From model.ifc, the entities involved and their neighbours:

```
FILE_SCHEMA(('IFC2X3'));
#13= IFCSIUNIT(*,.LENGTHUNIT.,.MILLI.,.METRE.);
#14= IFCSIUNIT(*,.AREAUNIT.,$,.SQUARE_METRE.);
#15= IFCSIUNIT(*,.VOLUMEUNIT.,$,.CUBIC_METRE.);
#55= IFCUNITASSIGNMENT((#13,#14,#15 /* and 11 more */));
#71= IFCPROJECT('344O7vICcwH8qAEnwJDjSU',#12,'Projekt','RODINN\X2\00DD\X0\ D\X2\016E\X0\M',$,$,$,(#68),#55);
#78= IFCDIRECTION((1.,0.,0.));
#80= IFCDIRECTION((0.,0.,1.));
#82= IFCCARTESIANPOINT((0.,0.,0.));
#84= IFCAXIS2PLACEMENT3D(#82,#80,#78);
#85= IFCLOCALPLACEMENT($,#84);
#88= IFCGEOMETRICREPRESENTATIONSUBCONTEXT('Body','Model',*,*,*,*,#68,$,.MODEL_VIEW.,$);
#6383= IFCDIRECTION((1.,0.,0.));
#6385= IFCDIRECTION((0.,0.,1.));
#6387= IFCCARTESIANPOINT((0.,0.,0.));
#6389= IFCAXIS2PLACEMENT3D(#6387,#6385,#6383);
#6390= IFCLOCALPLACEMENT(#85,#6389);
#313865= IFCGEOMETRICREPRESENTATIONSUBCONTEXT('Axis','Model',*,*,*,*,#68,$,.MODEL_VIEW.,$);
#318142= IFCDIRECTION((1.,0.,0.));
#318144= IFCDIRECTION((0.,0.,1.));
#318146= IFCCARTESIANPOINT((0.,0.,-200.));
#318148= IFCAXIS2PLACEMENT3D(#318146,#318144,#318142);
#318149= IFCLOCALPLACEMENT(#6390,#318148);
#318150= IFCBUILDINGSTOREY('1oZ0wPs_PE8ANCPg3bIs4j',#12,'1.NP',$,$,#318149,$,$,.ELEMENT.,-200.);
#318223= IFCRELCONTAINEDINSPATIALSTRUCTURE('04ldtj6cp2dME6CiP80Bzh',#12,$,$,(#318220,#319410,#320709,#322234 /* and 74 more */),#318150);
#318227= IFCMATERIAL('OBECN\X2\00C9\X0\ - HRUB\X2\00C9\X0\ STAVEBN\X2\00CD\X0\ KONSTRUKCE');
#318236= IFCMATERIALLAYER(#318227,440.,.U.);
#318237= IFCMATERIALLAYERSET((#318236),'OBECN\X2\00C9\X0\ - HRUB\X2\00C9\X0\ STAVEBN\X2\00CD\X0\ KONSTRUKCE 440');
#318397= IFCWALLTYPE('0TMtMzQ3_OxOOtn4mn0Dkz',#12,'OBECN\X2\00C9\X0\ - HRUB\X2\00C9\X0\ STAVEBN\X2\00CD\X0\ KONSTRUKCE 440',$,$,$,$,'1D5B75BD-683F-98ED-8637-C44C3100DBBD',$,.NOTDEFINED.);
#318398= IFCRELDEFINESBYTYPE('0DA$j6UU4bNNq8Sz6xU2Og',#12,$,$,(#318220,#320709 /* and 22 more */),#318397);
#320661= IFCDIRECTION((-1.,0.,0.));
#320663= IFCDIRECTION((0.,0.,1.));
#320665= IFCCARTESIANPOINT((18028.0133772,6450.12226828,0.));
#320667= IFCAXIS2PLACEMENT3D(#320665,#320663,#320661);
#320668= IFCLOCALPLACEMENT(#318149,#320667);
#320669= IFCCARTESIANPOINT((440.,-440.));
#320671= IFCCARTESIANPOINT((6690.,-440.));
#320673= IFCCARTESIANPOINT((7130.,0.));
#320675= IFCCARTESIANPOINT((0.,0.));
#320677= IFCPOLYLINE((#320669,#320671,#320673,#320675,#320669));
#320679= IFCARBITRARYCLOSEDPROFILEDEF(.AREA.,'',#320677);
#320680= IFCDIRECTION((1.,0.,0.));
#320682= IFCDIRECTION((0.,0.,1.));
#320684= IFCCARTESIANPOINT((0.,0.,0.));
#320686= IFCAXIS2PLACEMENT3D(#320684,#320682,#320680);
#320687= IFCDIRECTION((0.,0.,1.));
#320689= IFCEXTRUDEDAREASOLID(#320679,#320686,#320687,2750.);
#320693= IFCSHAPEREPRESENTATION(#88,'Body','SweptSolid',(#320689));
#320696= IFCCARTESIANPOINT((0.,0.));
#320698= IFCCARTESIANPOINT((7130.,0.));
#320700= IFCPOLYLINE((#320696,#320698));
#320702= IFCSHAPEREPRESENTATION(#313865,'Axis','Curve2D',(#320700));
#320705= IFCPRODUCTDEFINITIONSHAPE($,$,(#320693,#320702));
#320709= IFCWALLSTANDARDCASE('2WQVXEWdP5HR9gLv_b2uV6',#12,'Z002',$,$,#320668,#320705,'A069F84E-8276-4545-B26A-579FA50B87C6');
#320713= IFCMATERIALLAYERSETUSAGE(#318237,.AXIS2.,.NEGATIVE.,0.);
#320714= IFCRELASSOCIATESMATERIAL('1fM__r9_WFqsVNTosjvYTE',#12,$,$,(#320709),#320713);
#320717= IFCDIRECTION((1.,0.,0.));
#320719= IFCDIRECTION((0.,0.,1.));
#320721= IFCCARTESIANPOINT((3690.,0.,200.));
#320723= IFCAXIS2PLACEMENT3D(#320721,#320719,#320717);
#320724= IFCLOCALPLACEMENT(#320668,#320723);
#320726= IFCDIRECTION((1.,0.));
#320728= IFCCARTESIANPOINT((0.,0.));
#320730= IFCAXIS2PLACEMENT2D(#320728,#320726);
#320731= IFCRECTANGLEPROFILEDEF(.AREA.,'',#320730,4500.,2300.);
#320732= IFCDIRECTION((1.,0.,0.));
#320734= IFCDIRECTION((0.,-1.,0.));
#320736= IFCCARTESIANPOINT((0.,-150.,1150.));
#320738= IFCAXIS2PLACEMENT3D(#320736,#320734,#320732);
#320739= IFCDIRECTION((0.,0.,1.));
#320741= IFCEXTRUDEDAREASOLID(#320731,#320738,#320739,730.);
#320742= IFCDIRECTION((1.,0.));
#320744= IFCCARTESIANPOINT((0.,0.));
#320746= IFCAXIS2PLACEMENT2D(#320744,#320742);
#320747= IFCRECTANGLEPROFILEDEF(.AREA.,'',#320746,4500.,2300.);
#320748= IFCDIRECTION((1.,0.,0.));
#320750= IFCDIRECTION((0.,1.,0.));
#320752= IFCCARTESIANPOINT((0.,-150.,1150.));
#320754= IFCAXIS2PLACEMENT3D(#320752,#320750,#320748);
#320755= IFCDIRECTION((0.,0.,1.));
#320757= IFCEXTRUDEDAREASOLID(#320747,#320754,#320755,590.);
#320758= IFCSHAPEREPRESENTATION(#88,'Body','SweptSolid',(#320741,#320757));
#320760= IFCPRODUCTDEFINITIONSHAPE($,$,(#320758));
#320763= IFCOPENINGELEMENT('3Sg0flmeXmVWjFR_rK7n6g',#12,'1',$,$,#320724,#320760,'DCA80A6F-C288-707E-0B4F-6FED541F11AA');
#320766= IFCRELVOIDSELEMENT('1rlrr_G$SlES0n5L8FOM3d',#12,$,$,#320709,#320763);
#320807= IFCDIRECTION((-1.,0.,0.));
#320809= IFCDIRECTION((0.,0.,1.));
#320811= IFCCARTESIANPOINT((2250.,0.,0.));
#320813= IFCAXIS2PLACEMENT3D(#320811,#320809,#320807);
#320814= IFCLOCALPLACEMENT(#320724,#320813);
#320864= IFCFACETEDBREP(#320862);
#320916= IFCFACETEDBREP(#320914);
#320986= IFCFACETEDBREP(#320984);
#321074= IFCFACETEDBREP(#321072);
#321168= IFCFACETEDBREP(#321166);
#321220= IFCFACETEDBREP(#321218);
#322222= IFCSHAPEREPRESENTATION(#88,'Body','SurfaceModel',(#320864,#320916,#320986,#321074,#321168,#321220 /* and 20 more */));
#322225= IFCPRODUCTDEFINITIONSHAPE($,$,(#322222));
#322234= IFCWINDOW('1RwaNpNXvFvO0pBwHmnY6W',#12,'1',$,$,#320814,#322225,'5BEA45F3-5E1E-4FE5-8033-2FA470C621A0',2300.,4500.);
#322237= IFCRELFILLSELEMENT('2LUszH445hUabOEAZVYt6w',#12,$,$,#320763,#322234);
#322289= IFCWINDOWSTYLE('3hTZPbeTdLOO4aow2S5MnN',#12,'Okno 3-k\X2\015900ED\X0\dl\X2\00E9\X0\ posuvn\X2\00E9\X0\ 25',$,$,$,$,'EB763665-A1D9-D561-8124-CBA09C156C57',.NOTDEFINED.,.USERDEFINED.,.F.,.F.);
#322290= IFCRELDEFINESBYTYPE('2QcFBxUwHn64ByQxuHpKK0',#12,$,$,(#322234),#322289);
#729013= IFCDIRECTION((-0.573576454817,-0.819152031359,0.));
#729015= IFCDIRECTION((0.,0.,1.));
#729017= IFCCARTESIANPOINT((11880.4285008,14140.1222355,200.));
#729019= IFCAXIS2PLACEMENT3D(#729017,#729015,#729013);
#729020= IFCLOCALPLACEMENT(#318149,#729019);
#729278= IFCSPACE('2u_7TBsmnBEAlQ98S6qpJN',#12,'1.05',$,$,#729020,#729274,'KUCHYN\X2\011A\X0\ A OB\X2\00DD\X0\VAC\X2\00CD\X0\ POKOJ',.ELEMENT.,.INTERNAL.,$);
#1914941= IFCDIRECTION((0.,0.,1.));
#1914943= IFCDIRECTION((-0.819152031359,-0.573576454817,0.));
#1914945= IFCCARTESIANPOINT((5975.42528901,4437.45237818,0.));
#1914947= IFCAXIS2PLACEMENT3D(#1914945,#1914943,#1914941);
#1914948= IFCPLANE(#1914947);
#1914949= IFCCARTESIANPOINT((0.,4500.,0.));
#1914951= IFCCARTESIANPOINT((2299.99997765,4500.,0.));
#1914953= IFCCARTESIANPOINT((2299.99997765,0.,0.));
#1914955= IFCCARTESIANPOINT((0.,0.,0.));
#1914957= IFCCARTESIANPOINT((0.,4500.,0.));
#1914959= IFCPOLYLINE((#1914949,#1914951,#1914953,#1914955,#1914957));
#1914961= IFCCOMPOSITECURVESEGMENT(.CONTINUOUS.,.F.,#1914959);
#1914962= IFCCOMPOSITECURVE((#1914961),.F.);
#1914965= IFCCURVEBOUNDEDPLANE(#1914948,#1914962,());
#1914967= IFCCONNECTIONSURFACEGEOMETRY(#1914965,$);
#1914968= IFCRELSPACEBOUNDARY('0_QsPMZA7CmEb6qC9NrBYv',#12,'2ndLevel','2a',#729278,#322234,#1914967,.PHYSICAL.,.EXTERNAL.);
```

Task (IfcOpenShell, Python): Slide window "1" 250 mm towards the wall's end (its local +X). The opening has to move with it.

```python
import numpy as np
import ifcopenshell
import ifcopenshell.api.geometry
import ifcopenshell.util.placement
import ifcopenshell.util.unit

model = ifcopenshell.open("model.ifc")
unit_scale = ifcopenshell.util.unit.calculate_unit_scale(model)

window = model.by_guid("1RwaNpNXvFvO0pBwHmnY6W")
opening = window.FillsVoids[0].RelatingOpeningElement
wall = opening.VoidsElements[0].RelatingBuildingElement

wall_matrix = ifcopenshell.util.placement.get_local_placement(wall.ObjectPlacement)
shift = wall_matrix[:3, 0] * 0.25 / unit_scale
before = ifcopenshell.util.placement.get_local_placement(window.ObjectPlacement)[:3, 3].copy()

# The window is placed relative to its opening, so it follows when the opening moves.
matrix = ifcopenshell.util.placement.get_local_placement(opening.ObjectPlacement)
matrix[:3, 3] += shift
ifcopenshell.api.geometry.edit_object_placement(
    model, product=opening, matrix=matrix, is_si=False, should_transform_children=True
)

# Space boundary surfaces are stored in each space's coordinates; move them too.
for rel in window.ProvidesBoundaries:
    if not rel.ConnectionGeometry:
        continue
    surface = rel.ConnectionGeometry.SurfaceOnRelatingElement.BasisSurface
    space_matrix = ifcopenshell.util.placement.get_local_placement(rel.RelatingSpace.ObjectPlacement)
    point = np.array(surface.Position.Location.Coordinates) + space_matrix[:3, :3].T @ shift
    surface.Position = model.createIfcAxis2Placement3D(
        model.createIfcCartesianPoint(point.tolist()), surface.Position.Axis, surface.Position.RefDirection
    )

after = ifcopenshell.util.placement.get_local_placement(window.ObjectPlacement)[:3, 3]
print("window moved by", (after - before).round(3) + 0.0)

model.write("model_rev.ifc")
```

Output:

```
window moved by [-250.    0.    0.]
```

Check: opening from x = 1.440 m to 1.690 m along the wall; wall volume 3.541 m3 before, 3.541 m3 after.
